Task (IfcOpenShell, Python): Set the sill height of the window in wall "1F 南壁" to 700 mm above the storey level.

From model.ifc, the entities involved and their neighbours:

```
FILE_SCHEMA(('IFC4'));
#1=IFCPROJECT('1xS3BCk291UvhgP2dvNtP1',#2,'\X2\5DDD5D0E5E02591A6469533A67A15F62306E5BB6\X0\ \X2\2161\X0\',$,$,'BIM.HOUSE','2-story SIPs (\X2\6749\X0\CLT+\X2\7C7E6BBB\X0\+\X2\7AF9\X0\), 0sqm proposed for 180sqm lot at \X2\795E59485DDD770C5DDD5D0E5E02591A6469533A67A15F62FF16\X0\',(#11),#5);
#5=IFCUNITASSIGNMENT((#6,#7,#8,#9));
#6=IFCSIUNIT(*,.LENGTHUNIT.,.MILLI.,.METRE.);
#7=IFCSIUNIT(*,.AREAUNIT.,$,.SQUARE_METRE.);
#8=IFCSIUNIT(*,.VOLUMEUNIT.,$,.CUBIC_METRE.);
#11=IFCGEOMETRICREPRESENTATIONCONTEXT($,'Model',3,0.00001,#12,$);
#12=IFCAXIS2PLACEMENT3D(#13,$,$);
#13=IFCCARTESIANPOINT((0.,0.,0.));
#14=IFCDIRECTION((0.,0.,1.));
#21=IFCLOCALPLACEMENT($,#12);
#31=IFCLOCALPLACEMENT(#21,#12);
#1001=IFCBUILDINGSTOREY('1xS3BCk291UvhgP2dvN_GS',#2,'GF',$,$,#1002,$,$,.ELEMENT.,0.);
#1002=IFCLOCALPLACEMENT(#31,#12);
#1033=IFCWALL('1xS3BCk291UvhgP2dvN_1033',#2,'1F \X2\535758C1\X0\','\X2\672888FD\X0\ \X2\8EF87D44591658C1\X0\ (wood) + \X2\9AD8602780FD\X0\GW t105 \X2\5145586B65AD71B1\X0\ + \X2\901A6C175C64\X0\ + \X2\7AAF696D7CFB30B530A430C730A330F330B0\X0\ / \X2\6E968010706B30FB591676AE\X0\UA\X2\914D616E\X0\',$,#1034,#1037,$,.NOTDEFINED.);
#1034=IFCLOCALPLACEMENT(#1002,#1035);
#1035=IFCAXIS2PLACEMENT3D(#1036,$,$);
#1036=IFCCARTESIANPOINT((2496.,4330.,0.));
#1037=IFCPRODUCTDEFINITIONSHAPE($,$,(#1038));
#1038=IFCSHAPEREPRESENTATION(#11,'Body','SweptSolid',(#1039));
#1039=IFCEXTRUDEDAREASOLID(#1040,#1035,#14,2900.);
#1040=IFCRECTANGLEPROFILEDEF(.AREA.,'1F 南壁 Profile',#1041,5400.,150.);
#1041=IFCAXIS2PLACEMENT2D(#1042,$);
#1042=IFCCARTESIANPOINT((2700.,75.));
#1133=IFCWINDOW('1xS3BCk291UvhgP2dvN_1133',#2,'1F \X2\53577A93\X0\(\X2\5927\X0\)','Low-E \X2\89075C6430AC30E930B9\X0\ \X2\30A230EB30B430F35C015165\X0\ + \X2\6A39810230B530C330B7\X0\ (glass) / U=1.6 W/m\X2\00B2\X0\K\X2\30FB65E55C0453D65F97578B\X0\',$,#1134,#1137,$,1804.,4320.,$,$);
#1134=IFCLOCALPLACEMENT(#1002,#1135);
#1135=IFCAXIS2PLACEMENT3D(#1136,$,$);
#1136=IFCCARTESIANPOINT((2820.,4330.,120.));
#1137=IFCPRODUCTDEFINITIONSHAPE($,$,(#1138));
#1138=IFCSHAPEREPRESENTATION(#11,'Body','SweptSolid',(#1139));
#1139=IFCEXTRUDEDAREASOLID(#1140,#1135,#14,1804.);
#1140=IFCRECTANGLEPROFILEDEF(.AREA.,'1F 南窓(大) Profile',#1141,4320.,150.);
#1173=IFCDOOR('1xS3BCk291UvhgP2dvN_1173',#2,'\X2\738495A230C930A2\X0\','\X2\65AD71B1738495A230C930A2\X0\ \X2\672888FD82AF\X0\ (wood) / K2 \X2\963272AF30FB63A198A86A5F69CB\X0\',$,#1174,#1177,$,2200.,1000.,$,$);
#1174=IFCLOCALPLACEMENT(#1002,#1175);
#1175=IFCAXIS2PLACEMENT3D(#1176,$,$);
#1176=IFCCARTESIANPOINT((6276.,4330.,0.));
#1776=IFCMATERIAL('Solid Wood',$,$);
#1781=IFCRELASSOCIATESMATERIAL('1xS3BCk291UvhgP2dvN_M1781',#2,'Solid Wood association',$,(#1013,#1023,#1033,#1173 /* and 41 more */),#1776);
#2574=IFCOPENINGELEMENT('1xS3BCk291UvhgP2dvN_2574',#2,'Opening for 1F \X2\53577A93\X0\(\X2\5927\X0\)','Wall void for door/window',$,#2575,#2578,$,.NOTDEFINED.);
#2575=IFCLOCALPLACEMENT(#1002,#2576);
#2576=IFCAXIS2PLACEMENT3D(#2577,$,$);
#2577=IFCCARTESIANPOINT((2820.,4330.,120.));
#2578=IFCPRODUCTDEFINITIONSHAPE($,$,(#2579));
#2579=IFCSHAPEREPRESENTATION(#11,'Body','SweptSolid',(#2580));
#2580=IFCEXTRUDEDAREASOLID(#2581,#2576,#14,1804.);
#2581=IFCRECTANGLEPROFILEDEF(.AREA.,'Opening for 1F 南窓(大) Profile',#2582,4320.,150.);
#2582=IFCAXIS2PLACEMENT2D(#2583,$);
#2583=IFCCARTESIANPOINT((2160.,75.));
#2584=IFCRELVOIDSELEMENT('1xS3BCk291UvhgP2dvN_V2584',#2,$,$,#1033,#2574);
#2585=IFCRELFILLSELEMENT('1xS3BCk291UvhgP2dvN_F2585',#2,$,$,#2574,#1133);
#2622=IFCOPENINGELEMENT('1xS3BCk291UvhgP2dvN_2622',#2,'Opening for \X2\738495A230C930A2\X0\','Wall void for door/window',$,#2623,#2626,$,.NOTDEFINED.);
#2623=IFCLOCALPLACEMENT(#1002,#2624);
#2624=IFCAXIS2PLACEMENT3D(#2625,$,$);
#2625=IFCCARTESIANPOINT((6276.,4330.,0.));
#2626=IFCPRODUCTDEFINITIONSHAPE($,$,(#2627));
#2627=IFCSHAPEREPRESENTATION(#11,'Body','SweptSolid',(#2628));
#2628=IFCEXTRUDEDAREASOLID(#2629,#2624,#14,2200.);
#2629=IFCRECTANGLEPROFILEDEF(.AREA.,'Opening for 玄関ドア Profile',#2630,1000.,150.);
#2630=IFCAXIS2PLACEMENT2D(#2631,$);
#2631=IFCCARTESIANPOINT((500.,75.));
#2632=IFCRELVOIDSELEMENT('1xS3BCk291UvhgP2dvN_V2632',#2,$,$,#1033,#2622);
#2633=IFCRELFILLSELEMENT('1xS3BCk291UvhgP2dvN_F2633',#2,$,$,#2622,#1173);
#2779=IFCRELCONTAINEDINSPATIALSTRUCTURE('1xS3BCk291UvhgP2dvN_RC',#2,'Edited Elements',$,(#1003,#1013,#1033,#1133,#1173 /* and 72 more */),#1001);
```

```python
import numpy as np
import ifcopenshell
import ifcopenshell.api.geometry
import ifcopenshell.geom
import ifcopenshell.util.element
import ifcopenshell.util.placement
import ifcopenshell.util.shape
import ifcopenshell.util.unit

model = ifcopenshell.open("model.ifc")
unit_scale = ifcopenshell.util.unit.calculate_unit_scale(model)

window = model.by_guid("1xS3BCk291UvhgP2dvN_1133")
opening = window.FillsVoids[0].RelatingOpeningElement
storey = ifcopenshell.util.element.get_container(window, ifc_class="IfcBuildingStorey")
level = ifcopenshell.util.placement.get_local_placement(storey.ObjectPlacement)[2, 3]

# The opening's origin need not be at the sill, so measure its lowest point.
shape = ifcopenshell.geom.create_shape(ifcopenshell.geom.settings(), opening)
bottom = ifcopenshell.util.shape.get_shape_bottom_elevation(shape, shape.geometry) / unit_scale
dz = level + 700.0 - bottom

shift = np.array([0.0, 0.0, dz])
# The window is not placed relative to its opening, so move both.
for product in (opening, window):
    matrix = ifcopenshell.util.placement.get_local_placement(product.ObjectPlacement)
    matrix[:3, 3] += shift
    ifcopenshell.api.geometry.edit_object_placement(model, product=product, matrix=matrix, is_si=False)

print(f"moved by {dz * unit_scale:+.3f} m")

model.write("model_updated.ifc")
```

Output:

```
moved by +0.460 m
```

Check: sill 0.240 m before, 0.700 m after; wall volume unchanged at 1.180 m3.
